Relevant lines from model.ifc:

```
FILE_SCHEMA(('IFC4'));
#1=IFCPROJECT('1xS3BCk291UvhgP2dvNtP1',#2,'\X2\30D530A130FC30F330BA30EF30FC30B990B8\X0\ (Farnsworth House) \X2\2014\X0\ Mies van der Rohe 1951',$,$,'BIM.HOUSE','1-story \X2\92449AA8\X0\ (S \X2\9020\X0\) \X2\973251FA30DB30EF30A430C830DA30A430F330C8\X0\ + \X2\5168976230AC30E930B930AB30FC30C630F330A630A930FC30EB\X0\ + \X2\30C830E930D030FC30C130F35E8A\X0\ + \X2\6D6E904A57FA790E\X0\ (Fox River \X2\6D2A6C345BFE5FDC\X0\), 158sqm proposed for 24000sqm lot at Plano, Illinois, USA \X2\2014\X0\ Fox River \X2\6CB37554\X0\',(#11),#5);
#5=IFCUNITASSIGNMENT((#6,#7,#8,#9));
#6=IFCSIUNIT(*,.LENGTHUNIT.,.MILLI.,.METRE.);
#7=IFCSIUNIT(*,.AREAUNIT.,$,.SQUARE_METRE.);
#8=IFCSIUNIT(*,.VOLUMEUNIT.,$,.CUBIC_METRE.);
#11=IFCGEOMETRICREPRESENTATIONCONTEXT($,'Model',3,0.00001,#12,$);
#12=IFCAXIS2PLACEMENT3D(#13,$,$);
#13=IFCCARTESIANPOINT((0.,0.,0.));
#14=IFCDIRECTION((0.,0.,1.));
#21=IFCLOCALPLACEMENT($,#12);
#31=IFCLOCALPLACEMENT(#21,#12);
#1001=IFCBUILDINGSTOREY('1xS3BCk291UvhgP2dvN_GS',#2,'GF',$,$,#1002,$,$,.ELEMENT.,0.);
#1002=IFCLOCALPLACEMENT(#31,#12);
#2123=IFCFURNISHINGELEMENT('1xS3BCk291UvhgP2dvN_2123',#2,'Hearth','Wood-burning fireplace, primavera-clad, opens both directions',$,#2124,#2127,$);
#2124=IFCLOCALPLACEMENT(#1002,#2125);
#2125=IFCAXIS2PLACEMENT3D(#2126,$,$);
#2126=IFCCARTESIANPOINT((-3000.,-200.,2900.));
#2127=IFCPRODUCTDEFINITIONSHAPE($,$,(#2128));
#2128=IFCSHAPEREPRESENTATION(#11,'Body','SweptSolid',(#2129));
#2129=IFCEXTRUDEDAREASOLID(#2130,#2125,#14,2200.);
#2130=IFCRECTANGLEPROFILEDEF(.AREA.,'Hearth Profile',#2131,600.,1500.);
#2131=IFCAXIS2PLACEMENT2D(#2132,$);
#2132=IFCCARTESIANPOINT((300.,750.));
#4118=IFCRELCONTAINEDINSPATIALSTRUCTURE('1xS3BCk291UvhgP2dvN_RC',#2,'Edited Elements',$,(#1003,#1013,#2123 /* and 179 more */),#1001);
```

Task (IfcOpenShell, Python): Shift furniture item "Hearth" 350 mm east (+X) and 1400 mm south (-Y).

```python
import ifcopenshell
import ifcopenshell.api.geometry
import ifcopenshell.util.placement

model = ifcopenshell.open("model.ifc")

item = model.by_id(2123)
matrix = ifcopenshell.util.placement.get_local_placement(item.ObjectPlacement)
matrix[0, 3] += 350.0
matrix[1, 3] -= 1400.0
ifcopenshell.api.geometry.edit_object_placement(model, product=item, matrix=matrix, is_si=False)

print(ifcopenshell.util.placement.get_local_placement(item.ObjectPlacement).round(3) + 0.0)

model.write("model_updated.ifc")
```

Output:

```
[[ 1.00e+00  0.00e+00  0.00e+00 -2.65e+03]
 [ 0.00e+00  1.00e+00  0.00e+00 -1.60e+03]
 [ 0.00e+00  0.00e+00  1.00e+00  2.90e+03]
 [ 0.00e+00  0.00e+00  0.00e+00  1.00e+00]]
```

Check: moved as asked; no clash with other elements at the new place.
